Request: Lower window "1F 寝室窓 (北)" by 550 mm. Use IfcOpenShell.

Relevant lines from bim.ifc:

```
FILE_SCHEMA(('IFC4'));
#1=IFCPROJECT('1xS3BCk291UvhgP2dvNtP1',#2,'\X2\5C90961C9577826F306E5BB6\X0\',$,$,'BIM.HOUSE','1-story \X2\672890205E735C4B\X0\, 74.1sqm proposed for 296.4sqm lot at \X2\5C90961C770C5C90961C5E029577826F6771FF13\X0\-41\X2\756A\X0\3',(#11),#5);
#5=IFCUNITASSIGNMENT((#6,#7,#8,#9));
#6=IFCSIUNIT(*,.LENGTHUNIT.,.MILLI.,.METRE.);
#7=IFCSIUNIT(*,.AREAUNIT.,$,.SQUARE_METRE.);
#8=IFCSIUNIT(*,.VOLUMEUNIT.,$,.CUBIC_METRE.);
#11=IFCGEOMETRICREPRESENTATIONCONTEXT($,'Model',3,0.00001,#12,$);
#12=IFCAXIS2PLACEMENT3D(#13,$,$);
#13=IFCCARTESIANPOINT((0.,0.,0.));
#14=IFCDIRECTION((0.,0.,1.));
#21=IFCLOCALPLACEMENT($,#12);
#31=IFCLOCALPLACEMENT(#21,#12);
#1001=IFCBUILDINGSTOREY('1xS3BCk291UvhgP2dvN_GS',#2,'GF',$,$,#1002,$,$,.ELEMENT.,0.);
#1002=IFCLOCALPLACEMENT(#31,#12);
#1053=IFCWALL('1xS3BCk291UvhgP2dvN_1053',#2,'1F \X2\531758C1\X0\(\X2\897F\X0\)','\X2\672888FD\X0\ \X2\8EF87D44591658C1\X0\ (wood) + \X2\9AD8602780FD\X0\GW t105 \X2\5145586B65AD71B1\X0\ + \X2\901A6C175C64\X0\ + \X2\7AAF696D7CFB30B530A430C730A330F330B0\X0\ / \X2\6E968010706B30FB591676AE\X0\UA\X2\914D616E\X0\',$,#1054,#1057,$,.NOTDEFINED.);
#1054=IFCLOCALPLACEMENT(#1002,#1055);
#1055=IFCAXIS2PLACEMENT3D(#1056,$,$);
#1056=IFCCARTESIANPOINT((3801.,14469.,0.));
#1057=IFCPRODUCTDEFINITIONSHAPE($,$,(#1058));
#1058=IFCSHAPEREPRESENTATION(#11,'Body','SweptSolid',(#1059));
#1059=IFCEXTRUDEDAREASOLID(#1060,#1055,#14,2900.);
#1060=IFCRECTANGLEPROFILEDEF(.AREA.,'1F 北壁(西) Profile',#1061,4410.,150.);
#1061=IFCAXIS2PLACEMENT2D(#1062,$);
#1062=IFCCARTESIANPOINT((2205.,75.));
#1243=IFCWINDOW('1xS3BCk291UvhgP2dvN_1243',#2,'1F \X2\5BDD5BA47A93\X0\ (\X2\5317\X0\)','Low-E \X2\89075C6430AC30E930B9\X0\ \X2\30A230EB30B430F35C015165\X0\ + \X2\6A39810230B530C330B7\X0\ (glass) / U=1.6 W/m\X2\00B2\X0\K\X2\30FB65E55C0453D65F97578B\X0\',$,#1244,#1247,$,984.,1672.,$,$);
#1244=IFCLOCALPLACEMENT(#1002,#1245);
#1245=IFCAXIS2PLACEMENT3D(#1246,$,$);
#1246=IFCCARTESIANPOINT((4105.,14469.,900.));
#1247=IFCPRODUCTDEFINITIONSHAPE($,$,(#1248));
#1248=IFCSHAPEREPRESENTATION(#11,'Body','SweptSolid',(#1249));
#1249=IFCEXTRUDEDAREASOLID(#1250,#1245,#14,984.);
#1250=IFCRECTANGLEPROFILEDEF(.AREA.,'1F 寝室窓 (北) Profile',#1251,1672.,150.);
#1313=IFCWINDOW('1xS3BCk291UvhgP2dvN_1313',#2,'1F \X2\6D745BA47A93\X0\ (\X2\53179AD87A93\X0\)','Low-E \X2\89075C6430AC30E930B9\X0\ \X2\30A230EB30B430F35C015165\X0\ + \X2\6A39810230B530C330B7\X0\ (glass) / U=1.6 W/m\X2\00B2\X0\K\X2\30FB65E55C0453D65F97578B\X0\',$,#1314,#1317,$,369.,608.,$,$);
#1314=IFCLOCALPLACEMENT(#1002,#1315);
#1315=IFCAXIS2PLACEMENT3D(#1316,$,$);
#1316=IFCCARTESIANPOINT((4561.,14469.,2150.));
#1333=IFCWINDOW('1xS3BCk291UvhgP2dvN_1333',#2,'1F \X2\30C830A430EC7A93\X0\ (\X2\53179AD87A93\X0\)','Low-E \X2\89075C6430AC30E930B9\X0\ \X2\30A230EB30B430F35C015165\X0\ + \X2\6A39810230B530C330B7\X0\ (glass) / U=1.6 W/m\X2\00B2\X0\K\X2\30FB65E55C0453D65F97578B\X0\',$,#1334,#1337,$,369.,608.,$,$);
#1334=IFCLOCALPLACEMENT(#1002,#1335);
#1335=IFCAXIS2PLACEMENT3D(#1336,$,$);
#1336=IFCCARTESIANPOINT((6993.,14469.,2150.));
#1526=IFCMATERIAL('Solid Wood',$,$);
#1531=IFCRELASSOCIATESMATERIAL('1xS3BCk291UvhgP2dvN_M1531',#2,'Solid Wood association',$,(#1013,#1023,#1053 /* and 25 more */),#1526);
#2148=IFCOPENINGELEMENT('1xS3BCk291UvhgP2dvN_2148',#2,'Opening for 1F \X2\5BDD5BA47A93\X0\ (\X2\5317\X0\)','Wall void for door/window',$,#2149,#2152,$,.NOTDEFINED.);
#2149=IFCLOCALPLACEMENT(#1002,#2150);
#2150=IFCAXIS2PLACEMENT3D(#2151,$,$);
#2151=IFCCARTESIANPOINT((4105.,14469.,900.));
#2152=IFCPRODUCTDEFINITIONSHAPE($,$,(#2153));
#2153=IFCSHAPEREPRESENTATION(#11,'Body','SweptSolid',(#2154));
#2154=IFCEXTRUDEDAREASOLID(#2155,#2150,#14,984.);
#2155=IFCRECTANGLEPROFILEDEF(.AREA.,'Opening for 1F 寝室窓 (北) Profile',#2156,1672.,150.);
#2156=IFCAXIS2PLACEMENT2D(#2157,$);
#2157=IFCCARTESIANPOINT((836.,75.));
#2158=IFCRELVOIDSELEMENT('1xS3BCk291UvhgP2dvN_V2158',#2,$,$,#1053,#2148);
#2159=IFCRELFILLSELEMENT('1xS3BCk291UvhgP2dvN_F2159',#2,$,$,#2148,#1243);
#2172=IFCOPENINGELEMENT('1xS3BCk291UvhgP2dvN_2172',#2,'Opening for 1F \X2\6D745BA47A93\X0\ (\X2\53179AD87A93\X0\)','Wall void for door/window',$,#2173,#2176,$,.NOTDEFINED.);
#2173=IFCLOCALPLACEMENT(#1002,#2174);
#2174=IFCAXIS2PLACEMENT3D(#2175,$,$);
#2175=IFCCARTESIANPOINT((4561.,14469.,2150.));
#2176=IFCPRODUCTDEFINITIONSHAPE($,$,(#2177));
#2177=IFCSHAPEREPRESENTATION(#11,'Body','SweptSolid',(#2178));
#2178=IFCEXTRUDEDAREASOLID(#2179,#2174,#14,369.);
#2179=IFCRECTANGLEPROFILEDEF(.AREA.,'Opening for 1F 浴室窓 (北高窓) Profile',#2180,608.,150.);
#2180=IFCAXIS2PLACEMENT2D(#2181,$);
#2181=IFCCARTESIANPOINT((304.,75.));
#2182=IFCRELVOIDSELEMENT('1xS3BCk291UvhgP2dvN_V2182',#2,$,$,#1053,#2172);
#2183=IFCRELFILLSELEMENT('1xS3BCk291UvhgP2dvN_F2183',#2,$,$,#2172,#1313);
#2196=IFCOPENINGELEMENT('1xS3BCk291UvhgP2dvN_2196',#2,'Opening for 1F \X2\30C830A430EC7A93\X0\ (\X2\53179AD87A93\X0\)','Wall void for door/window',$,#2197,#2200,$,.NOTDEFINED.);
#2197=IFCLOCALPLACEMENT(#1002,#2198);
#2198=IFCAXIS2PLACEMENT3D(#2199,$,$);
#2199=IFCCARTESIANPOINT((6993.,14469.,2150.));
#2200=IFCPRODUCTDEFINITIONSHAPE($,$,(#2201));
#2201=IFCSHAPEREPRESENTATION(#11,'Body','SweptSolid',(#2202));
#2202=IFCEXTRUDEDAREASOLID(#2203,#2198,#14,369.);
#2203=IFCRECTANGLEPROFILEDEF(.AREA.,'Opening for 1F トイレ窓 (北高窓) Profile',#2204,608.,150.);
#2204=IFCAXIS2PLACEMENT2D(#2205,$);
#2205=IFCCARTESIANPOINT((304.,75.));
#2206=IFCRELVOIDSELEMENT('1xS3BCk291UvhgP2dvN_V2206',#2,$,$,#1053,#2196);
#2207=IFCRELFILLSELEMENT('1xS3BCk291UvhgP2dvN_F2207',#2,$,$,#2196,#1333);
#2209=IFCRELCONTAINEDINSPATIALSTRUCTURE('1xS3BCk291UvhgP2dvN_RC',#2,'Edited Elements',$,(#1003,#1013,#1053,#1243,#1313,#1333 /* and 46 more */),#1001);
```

```python
import numpy as np
import ifcopenshell
import ifcopenshell.api.geometry
import ifcopenshell.util.placement
import ifcopenshell.util.unit

model = ifcopenshell.open("bim.ifc")
unit_scale = ifcopenshell.util.unit.calculate_unit_scale(model)

window = model.by_id(1243)
opening = window.FillsVoids[0].RelatingOpeningElement
dz = -0.55 / unit_scale

shift = np.array([0.0, 0.0, dz])
# The window is not placed relative to its opening, so move both.
for product in (opening, window):
    matrix = ifcopenshell.util.placement.get_local_placement(product.ObjectPlacement)
    matrix[:3, 3] += shift
    ifcopenshell.api.geometry.edit_object_placement(model, product=product, matrix=matrix, is_si=False)

print(f"moved by {dz * unit_scale:+.3f} m")

model.write("bim_updated.ifc")
```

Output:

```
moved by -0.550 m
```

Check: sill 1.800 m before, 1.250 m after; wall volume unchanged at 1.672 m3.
